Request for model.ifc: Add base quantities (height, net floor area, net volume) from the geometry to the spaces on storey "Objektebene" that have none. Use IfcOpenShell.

First a look at what the model holds.

```python
import ifcopenshell
import ifcopenshell.util.element
import ifcopenshell.util.unit

model = ifcopenshell.open("model.ifc")
print(model.schema)
for unit_type in ("LENGTHUNIT", "AREAUNIT", "VOLUMEUNIT"):
    print(unit_type, ifcopenshell.util.unit.calculate_unit_scale(model, unit_type))
storey = next(s for s in model.by_type("IfcBuildingStorey") if s.Name == "Objektebene")
spaces = [e for e in ifcopenshell.util.element.get_decomposition(storey) if e.is_a("IfcSpace")]
for e in sorted(spaces, key=lambda e: e.id()):
    print(e.id(), e.is_a(), e.Name, list(ifcopenshell.util.element.get_psets(e, qtos_only=True)), sep=" | ")
```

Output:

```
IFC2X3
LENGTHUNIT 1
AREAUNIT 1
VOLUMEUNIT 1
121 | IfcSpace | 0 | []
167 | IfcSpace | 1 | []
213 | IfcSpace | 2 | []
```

```python
import ifcopenshell
import ifcopenshell.api.pset
import ifcopenshell.geom
import ifcopenshell.util.element
import ifcopenshell.util.shape
import ifcopenshell.util.unit

model = ifcopenshell.open("model.ifc")
unit_scale = ifcopenshell.util.unit.calculate_unit_scale(model)
area_scale = ifcopenshell.util.unit.calculate_unit_scale(model, "AREAUNIT")
volume_scale = ifcopenshell.util.unit.calculate_unit_scale(model, "VOLUMEUNIT")
settings = ifcopenshell.geom.settings()

storey = next(s for s in model.by_type("IfcBuildingStorey") if s.Name == "Objektebene")
spaces = [e for e in ifcopenshell.util.element.get_decomposition(storey) if e.is_a("IfcSpace")]

for e in sorted(spaces, key=lambda e: e.id()):
    if ifcopenshell.util.element.get_psets(e, qtos_only=True, should_inherit=False):
        continue
    # Geometry comes back in metres, in the element's own axes.
    shape = ifcopenshell.geom.create_shape(settings, e)
    values = {
        "Height": ifcopenshell.util.shape.get_z(shape.geometry) / unit_scale,
        "NetFloorArea": ifcopenshell.util.shape.get_footprint_area(shape.geometry) / area_scale,
        "NetVolume": ifcopenshell.util.shape.get_volume(shape.geometry) / volume_scale,
    }
    qto = ifcopenshell.api.pset.add_qto(model, product=e, name="BaseQuantities")
    ifcopenshell.api.pset.edit_qto(model, qto=qto, properties=values)
    print(e.id(), {k: round(v, 3) for k, v in values.items()})

model.write("model-out.ifc")
```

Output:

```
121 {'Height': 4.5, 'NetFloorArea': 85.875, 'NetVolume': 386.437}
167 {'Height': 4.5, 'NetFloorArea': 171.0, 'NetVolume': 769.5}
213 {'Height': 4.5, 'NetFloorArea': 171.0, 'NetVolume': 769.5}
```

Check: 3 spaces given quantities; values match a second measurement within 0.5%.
